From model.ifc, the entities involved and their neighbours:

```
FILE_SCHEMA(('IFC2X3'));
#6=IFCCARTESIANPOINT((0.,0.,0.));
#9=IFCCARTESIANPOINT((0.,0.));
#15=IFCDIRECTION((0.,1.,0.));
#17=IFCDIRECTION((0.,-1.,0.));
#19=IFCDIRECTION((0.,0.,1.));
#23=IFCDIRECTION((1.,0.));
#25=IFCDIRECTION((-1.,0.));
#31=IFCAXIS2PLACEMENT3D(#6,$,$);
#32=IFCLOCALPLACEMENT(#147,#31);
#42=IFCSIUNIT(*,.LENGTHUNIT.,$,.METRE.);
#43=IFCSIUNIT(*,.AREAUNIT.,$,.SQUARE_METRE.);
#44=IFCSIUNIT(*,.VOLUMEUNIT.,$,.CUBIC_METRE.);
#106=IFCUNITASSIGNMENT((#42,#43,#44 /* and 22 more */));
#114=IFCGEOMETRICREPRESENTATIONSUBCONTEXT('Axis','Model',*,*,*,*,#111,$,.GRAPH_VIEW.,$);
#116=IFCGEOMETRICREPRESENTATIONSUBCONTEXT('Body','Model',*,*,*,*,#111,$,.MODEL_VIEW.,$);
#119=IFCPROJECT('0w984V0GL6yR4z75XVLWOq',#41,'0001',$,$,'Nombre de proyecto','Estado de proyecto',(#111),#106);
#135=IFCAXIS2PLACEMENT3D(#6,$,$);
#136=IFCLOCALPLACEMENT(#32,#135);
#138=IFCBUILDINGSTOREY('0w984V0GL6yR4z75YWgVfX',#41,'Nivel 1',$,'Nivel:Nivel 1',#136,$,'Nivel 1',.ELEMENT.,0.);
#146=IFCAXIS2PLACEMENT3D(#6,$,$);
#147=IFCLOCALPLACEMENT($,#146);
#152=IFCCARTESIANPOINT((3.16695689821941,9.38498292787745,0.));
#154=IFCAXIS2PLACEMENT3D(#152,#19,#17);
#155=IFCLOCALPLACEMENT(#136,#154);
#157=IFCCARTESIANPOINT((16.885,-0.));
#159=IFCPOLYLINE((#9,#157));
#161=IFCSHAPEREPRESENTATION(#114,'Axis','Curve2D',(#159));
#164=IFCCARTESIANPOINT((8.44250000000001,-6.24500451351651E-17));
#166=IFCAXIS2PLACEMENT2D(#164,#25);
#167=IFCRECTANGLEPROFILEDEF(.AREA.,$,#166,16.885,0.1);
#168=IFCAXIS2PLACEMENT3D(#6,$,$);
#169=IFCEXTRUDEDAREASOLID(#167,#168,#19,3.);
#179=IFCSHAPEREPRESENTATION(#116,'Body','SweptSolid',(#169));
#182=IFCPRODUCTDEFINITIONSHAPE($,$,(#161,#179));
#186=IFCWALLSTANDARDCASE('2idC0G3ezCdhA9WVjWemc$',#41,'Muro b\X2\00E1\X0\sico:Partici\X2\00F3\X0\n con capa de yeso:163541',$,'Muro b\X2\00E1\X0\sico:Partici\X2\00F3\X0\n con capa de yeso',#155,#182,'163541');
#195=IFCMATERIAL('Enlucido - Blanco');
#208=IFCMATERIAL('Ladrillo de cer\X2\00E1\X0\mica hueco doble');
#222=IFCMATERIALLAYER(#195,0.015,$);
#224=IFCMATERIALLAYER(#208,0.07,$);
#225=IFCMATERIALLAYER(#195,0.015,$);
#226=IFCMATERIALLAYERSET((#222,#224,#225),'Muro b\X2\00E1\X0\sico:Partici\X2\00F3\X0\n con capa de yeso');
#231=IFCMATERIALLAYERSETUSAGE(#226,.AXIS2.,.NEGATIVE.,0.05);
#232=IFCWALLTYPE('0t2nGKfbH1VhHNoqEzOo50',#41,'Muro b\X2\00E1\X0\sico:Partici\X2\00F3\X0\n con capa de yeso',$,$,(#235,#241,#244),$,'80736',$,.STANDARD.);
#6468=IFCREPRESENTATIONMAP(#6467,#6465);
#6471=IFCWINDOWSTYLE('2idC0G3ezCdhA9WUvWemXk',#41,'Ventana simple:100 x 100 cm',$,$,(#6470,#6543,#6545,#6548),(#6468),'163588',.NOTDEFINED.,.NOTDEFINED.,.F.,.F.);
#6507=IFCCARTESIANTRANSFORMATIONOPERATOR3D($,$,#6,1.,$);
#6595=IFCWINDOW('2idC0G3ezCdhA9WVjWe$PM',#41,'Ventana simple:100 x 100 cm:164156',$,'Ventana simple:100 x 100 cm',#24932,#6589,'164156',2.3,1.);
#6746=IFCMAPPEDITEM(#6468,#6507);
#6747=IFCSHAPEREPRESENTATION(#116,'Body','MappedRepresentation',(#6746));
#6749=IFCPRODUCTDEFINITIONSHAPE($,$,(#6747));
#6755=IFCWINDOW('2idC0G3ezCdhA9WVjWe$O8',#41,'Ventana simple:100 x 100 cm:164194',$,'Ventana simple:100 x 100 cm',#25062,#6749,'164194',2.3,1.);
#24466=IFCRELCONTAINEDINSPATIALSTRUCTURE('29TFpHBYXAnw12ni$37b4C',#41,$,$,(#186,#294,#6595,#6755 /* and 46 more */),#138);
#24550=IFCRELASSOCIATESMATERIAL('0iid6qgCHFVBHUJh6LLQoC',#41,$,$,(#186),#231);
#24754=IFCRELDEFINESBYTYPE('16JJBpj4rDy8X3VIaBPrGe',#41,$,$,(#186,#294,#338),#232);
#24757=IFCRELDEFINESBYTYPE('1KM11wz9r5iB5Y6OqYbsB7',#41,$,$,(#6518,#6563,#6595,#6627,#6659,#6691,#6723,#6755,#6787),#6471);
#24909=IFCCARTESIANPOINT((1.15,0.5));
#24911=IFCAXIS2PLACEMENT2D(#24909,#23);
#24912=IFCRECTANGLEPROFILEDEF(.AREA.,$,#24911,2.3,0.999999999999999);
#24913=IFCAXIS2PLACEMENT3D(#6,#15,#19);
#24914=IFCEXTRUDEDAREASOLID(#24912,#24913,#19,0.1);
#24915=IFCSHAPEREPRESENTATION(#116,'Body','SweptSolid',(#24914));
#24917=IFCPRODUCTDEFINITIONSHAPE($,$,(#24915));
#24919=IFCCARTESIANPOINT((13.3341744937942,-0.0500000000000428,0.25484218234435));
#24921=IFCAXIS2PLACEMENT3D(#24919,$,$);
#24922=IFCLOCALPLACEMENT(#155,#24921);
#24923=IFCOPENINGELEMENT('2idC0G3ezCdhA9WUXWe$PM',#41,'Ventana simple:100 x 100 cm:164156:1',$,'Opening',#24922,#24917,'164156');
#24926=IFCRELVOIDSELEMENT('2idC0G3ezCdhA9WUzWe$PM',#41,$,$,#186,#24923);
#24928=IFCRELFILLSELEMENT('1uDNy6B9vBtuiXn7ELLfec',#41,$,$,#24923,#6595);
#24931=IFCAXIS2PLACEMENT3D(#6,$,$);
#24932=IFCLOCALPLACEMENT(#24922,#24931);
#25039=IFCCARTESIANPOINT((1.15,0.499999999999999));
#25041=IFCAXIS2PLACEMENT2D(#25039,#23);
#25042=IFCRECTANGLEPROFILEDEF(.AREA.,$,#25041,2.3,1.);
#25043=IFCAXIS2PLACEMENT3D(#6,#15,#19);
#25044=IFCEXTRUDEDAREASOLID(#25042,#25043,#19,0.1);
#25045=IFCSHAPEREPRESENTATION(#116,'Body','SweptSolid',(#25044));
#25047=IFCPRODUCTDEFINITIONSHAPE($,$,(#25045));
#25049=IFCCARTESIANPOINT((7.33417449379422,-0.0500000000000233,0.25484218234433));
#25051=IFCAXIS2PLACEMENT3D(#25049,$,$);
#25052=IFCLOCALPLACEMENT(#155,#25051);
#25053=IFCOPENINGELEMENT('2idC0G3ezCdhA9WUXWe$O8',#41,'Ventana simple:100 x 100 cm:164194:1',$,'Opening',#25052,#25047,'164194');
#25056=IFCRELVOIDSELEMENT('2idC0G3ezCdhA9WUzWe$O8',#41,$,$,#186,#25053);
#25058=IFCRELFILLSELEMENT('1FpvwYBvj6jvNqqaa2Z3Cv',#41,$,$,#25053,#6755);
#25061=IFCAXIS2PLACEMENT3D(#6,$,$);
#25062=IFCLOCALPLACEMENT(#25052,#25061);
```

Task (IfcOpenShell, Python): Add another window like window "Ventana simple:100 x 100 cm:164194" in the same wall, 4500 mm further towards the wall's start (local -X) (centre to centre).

```python
import ifcopenshell
import ifcopenshell.api.feature
import ifcopenshell.api.geometry
import ifcopenshell.api.root
import ifcopenshell.geom
import ifcopenshell.util.element
import ifcopenshell.util.placement
import ifcopenshell.util.shape

model = ifcopenshell.open("model.ifc")
settings = ifcopenshell.geom.settings()


def volume(element):
    """Net volume in cubic metres, openings subtracted."""
    shape = ifcopenshell.geom.create_shape(settings, element)
    return ifcopenshell.util.shape.get_volume(shape.geometry)


def reuse_history(source, copy):
    """copy_class also copies each property set's owner history, people and application; keep the originals."""
    for rel in copy.IsDefinedBy:
        if rel.is_a("IfcRelDefinesByProperties") and (history := rel.RelatingPropertyDefinition.OwnerHistory):
            rel.RelatingPropertyDefinition.OwnerHistory = source.OwnerHistory
            ifcopenshell.util.element.remove_deep2(model, history)


window = model.by_id(6755)
opening = window.FillsVoids[0].RelatingOpeningElement
wall = opening.VoidsElements[0].RelatingBuildingElement
before = volume(wall)
shift = ifcopenshell.util.placement.get_local_placement(wall.ObjectPlacement)[:3, 0] * -4.5

# copy_class copies the void relationship, type, container and properties, but no geometry.
new_opening = ifcopenshell.api.root.copy_class(model, product=opening)
new_opening.Representation = ifcopenshell.util.element.copy_deep(
    model, opening.Representation, exclude=["IfcGeometricRepresentationContext", "IfcRepresentationMap"]
)
new_opening.Name = "Ventana simple:100 x 100 cm"
new_opening.Tag = None
new_window = ifcopenshell.api.root.copy_class(model, product=window)
new_window.Representation = ifcopenshell.util.element.copy_deep(
    model, window.Representation, exclude=["IfcGeometricRepresentationContext", "IfcRepresentationMap"]
)
new_window.Name = "Ventana simple:100 x 100 cm"
new_window.Tag = None
reuse_history(window, new_window)
fills = ifcopenshell.api.feature.add_filling(model, opening=new_opening, element=new_window)
fills.OwnerHistory = new_window.OwnerHistory  # required in IFC2X3

for old, new in ((opening, new_opening), (window, new_window)):
    matrix = ifcopenshell.util.placement.get_local_placement(old.ObjectPlacement)
    matrix[:3, 3] += shift
    ifcopenshell.api.geometry.edit_object_placement(model, product=new, matrix=matrix, is_si=False)

after = volume(wall)

print(f"wall volume {before:.3f} -> {after:.3f} m3")

model.write("model_updated.ifc")
```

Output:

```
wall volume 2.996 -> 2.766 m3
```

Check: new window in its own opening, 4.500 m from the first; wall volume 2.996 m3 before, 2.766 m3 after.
